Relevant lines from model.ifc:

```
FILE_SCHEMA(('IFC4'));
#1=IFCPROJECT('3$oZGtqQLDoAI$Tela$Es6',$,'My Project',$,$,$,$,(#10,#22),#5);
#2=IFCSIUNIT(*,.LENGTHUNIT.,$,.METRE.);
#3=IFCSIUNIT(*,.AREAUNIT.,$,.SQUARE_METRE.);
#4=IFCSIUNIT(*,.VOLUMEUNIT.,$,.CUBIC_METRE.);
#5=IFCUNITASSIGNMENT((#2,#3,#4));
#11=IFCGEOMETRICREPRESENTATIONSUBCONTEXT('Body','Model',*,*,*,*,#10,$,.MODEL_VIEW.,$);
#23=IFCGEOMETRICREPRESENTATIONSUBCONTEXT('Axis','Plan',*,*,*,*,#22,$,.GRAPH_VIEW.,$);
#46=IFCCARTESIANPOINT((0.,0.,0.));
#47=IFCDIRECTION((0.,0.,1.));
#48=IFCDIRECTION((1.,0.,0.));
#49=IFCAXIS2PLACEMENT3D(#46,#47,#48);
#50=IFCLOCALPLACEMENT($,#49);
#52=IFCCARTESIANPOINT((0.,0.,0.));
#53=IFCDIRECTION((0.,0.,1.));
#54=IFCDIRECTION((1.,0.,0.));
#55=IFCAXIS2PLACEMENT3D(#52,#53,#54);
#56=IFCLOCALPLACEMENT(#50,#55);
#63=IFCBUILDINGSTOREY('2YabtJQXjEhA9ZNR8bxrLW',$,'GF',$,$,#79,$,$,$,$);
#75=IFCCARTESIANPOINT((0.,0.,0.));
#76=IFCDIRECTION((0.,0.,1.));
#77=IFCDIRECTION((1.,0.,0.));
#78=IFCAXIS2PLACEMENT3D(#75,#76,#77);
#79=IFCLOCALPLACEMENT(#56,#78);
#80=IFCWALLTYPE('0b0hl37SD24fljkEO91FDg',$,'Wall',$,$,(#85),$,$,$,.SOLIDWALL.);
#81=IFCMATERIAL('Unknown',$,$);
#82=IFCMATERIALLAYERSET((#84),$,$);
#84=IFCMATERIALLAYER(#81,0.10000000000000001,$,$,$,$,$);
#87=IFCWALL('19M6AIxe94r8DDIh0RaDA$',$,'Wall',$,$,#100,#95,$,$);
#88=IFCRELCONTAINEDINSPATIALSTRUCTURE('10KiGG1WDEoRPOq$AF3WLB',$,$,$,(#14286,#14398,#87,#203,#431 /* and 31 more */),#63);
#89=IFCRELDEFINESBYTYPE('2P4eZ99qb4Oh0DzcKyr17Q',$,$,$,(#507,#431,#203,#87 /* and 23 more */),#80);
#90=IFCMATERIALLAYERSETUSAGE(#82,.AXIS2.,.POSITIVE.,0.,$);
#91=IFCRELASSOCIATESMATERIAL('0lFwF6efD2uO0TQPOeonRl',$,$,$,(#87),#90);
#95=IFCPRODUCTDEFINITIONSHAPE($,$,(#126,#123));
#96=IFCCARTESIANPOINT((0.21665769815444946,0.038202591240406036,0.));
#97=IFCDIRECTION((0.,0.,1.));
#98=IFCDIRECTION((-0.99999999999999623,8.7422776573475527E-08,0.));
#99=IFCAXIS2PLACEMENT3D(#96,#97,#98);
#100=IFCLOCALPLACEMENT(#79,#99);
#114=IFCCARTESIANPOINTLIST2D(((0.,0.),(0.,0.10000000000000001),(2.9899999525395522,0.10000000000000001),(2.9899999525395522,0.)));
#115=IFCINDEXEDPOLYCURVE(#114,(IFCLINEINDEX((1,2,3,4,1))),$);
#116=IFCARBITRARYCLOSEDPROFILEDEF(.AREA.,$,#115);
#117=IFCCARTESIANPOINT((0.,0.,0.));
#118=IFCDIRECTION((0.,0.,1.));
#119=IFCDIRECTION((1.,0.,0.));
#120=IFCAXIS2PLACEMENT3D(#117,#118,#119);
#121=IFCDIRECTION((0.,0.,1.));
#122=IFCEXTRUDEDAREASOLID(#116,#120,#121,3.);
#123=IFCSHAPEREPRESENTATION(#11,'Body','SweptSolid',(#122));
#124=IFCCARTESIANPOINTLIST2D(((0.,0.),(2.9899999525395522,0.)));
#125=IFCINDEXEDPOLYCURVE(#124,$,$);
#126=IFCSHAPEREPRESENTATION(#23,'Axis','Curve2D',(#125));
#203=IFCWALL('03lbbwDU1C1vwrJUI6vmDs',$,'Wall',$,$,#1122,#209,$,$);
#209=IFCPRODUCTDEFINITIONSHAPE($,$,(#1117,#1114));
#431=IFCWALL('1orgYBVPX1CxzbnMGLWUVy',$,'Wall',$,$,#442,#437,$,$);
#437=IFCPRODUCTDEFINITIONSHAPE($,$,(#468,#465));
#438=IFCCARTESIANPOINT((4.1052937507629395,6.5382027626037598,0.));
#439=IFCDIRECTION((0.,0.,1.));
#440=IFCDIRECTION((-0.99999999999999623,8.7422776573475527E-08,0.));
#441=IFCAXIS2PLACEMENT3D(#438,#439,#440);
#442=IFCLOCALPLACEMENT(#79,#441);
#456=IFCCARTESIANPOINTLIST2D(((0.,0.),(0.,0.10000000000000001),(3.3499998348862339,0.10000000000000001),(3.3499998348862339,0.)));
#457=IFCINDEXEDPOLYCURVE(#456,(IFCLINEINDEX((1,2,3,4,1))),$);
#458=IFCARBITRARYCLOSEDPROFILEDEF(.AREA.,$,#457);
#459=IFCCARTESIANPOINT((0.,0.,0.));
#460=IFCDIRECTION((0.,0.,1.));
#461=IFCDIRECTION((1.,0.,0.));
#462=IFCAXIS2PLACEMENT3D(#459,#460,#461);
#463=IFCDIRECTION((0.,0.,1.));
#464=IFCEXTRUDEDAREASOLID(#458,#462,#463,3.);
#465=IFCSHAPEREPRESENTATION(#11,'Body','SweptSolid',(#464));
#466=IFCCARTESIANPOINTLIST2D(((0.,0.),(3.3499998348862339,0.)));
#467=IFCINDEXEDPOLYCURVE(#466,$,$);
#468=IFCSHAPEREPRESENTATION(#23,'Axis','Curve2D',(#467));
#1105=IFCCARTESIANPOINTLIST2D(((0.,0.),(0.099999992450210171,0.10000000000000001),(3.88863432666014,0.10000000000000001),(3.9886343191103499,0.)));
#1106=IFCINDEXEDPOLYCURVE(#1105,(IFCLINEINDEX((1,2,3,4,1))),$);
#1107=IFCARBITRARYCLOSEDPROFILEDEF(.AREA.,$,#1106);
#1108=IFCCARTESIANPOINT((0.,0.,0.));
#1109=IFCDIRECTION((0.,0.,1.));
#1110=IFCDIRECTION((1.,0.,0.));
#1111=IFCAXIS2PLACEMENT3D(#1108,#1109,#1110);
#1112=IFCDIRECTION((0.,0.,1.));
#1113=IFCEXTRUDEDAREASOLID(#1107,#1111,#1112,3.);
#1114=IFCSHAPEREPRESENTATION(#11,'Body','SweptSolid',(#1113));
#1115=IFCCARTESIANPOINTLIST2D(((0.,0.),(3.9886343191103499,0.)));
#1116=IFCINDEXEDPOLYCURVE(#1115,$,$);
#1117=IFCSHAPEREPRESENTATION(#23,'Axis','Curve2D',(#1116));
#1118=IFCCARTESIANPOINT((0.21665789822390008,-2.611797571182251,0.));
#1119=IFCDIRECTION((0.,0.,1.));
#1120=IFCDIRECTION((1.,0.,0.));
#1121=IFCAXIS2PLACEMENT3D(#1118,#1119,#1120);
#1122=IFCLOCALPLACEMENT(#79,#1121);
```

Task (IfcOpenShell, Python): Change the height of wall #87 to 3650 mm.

```python
import ifcopenshell
import ifcopenshell.geom
import ifcopenshell.util.representation
import ifcopenshell.util.shape
import ifcopenshell.util.unit

model = ifcopenshell.open("model.ifc")
unit_scale = ifcopenshell.util.unit.calculate_unit_scale(model)
settings = ifcopenshell.geom.settings()


def volume(element):
    """Net volume in cubic metres, openings subtracted."""
    shape = ifcopenshell.geom.create_shape(settings, element)
    return ifcopenshell.util.shape.get_volume(shape.geometry)


wall = model.by_guid("19M6AIxe94r8DDIh0RaDA$")
before = volume(wall)

body = ifcopenshell.util.representation.get_representation(wall, "Model", "Body")
solid = body.Items[0]
old_height = solid.Depth
solid.Depth = 3.65 / unit_scale
after = volume(wall)

print(f"height {old_height:g} -> {solid.Depth:g}, volume {before:.3f} -> {after:.3f} m3")

model.write("model_v2.ifc")
```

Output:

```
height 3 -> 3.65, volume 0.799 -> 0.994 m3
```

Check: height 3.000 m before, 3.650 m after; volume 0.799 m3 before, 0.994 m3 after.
